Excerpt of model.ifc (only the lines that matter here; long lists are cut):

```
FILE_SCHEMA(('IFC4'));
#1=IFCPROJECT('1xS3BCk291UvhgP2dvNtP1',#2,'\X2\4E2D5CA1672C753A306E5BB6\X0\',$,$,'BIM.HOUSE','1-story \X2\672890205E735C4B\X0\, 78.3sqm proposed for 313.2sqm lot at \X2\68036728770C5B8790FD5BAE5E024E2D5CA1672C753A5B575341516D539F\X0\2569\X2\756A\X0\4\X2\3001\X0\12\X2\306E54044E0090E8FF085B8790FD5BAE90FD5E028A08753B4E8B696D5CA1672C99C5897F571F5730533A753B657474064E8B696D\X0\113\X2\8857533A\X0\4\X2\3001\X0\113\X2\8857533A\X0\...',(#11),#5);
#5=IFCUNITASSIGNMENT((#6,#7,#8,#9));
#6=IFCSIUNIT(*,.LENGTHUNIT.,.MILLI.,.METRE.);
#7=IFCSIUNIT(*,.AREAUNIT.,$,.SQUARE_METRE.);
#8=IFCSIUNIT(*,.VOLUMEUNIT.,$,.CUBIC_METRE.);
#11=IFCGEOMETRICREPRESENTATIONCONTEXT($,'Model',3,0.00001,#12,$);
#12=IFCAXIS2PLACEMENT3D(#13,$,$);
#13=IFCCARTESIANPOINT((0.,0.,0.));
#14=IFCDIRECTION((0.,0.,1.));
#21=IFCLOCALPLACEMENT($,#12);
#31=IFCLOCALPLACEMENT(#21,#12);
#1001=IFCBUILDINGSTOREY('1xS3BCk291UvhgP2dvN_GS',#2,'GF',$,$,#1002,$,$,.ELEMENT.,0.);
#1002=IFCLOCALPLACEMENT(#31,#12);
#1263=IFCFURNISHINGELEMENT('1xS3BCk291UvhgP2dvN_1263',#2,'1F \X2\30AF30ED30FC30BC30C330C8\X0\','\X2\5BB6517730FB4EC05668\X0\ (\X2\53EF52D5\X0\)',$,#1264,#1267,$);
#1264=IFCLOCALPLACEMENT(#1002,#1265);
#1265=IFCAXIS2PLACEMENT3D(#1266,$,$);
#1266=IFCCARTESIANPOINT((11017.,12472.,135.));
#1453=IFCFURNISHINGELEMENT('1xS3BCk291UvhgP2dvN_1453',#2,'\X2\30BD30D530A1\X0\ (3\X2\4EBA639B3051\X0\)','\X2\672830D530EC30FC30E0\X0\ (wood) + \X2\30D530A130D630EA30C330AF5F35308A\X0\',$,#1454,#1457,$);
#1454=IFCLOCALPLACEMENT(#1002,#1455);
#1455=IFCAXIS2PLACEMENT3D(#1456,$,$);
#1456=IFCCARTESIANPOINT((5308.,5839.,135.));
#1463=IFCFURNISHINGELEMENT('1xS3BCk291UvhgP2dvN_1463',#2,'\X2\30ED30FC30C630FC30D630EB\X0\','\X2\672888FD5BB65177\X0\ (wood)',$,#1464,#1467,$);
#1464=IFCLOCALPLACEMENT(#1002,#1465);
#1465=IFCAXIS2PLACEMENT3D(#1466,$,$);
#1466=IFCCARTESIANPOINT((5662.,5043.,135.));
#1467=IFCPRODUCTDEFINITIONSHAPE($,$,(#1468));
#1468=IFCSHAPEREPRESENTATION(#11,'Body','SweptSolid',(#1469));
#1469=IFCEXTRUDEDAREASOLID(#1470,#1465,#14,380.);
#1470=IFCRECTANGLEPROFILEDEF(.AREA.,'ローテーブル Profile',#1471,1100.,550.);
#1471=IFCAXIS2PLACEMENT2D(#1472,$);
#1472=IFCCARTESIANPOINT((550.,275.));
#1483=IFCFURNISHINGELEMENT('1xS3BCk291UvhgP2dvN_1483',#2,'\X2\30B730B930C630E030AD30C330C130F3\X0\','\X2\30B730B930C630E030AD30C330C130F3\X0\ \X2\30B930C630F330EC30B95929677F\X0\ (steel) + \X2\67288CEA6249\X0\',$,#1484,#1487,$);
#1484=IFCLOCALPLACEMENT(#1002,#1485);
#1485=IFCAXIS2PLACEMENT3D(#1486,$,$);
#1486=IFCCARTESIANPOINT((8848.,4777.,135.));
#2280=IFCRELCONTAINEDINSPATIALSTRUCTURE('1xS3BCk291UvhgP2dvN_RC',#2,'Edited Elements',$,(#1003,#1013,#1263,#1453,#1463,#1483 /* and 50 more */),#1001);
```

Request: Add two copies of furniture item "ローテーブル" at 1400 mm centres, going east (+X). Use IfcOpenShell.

```python
import numpy as np
import ifcopenshell
import ifcopenshell.api.geometry
import ifcopenshell.api.root
import ifcopenshell.util.element
import ifcopenshell.util.placement
import ifcopenshell.util.unit

model = ifcopenshell.open("model.ifc")
unit_scale = ifcopenshell.util.unit.calculate_unit_scale(model)


def reuse_history(source, copy):
    """copy_class also copies each property set's owner history, people and application; keep the originals."""
    for rel in copy.IsDefinedBy:
        if rel.is_a("IfcRelDefinesByProperties") and (history := rel.RelatingPropertyDefinition.OwnerHistory):
            rel.RelatingPropertyDefinition.OwnerHistory = source.OwnerHistory
            ifcopenshell.util.element.remove_deep2(model, history)


source = model.by_guid("1xS3BCk291UvhgP2dvN_1463")
base = ifcopenshell.util.placement.get_local_placement(source.ObjectPlacement)
step = np.array([1.0, 0.0, 0.0]) * 1.4 / unit_scale

for i in range(1, 3):
    copy = ifcopenshell.api.root.copy_class(model, product=source)
    copy.Representation = ifcopenshell.util.element.copy_deep(
        model, source.Representation, exclude=["IfcGeometricRepresentationContext", "IfcRepresentationMap"]
    )
    reuse_history(source, copy)
    matrix = base.copy()
    matrix[:3, 3] += i * step
    print("added at", matrix[:3, 3].round(3) + 0.0)
    ifcopenshell.api.geometry.edit_object_placement(model, product=copy, matrix=matrix, is_si=False)

model.write("model_rev.ifc")
```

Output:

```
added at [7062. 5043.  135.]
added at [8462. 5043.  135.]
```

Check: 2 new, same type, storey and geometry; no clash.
